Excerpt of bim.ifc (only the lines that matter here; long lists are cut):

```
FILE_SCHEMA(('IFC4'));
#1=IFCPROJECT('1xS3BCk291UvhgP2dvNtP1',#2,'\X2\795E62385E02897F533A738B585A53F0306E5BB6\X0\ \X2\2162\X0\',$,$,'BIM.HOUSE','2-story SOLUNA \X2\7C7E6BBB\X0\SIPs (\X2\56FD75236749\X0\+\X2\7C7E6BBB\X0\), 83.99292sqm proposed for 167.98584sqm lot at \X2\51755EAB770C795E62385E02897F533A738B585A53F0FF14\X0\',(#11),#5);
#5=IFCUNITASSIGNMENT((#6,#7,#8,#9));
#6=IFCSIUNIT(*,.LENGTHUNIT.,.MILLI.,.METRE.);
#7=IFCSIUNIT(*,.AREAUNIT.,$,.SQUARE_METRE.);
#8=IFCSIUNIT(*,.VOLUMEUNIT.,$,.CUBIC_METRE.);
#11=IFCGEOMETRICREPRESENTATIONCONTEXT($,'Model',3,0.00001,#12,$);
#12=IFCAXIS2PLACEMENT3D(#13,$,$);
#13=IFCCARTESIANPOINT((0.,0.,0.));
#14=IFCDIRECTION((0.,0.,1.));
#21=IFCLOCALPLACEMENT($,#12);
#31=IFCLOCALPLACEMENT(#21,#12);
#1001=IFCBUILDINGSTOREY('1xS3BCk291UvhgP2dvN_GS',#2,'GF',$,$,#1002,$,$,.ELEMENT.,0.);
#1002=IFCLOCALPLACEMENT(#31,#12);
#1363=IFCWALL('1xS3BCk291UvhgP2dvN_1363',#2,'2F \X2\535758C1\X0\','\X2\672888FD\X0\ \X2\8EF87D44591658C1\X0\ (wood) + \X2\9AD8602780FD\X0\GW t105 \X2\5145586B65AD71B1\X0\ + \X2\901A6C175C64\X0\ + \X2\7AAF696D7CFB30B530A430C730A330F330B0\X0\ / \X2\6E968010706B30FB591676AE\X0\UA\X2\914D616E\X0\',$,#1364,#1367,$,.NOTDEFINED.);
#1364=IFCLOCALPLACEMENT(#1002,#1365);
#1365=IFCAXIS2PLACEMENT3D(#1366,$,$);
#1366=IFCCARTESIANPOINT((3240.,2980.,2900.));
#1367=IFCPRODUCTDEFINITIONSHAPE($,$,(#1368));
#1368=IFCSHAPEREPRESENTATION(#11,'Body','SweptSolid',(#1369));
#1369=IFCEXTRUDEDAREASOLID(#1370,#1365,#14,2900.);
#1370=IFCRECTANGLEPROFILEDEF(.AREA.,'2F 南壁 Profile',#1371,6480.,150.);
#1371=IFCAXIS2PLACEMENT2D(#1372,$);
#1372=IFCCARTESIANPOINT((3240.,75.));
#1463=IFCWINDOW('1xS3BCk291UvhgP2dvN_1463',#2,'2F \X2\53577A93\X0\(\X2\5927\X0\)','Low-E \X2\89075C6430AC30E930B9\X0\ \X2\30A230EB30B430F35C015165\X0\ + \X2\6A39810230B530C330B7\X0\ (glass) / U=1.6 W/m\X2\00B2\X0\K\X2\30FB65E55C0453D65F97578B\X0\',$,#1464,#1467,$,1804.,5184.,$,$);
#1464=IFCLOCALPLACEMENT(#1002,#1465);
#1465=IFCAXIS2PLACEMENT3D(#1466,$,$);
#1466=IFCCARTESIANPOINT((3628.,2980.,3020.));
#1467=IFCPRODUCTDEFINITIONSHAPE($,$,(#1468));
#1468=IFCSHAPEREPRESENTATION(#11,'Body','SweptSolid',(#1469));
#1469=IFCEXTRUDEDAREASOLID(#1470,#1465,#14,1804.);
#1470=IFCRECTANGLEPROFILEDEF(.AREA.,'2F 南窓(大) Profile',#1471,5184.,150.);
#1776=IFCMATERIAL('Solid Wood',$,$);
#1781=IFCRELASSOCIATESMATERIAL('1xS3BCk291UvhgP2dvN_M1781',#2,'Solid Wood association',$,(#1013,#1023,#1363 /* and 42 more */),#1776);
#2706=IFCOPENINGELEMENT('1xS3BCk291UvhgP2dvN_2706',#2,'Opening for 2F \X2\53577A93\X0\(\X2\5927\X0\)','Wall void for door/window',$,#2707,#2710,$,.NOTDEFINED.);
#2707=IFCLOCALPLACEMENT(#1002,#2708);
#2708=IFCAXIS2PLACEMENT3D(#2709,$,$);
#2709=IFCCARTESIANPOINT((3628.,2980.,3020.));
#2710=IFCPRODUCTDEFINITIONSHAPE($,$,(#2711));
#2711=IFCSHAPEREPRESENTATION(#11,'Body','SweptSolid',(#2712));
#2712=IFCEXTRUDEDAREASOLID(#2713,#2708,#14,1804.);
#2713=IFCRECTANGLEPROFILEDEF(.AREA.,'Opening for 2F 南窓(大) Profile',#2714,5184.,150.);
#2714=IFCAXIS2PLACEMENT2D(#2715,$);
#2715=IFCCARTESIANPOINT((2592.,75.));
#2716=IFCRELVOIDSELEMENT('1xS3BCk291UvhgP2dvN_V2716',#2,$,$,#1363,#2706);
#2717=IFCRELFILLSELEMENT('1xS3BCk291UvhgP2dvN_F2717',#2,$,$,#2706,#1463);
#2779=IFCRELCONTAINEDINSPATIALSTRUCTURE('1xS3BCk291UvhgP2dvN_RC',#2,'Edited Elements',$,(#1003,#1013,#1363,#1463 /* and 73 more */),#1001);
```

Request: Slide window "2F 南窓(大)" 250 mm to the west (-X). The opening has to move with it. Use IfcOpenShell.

```python
import ifcopenshell
import ifcopenshell.api.geometry
import ifcopenshell.util.placement

model = ifcopenshell.open("bim.ifc")

window = model.by_guid("1xS3BCk291UvhgP2dvN_1463")
opening = window.FillsVoids[0].RelatingOpeningElement
wall = opening.VoidsElements[0].RelatingBuildingElement

wall_matrix = ifcopenshell.util.placement.get_local_placement(wall.ObjectPlacement)
shift = wall_matrix[:3, 0] * -250.0
before = ifcopenshell.util.placement.get_local_placement(window.ObjectPlacement)[:3, 3].copy()

# The window is not placed relative to its opening, so move both.
for product in (opening, window):
    matrix = ifcopenshell.util.placement.get_local_placement(product.ObjectPlacement)
    matrix[:3, 3] += shift
    ifcopenshell.api.geometry.edit_object_placement(model, product=product, matrix=matrix, is_si=False)

after = ifcopenshell.util.placement.get_local_placement(window.ObjectPlacement)[:3, 3]
print("window moved by", (after - before).round(3) + 0.0)

model.write("bim_updated.ifc")
```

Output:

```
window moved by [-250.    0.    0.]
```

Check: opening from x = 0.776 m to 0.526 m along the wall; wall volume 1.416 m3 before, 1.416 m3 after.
